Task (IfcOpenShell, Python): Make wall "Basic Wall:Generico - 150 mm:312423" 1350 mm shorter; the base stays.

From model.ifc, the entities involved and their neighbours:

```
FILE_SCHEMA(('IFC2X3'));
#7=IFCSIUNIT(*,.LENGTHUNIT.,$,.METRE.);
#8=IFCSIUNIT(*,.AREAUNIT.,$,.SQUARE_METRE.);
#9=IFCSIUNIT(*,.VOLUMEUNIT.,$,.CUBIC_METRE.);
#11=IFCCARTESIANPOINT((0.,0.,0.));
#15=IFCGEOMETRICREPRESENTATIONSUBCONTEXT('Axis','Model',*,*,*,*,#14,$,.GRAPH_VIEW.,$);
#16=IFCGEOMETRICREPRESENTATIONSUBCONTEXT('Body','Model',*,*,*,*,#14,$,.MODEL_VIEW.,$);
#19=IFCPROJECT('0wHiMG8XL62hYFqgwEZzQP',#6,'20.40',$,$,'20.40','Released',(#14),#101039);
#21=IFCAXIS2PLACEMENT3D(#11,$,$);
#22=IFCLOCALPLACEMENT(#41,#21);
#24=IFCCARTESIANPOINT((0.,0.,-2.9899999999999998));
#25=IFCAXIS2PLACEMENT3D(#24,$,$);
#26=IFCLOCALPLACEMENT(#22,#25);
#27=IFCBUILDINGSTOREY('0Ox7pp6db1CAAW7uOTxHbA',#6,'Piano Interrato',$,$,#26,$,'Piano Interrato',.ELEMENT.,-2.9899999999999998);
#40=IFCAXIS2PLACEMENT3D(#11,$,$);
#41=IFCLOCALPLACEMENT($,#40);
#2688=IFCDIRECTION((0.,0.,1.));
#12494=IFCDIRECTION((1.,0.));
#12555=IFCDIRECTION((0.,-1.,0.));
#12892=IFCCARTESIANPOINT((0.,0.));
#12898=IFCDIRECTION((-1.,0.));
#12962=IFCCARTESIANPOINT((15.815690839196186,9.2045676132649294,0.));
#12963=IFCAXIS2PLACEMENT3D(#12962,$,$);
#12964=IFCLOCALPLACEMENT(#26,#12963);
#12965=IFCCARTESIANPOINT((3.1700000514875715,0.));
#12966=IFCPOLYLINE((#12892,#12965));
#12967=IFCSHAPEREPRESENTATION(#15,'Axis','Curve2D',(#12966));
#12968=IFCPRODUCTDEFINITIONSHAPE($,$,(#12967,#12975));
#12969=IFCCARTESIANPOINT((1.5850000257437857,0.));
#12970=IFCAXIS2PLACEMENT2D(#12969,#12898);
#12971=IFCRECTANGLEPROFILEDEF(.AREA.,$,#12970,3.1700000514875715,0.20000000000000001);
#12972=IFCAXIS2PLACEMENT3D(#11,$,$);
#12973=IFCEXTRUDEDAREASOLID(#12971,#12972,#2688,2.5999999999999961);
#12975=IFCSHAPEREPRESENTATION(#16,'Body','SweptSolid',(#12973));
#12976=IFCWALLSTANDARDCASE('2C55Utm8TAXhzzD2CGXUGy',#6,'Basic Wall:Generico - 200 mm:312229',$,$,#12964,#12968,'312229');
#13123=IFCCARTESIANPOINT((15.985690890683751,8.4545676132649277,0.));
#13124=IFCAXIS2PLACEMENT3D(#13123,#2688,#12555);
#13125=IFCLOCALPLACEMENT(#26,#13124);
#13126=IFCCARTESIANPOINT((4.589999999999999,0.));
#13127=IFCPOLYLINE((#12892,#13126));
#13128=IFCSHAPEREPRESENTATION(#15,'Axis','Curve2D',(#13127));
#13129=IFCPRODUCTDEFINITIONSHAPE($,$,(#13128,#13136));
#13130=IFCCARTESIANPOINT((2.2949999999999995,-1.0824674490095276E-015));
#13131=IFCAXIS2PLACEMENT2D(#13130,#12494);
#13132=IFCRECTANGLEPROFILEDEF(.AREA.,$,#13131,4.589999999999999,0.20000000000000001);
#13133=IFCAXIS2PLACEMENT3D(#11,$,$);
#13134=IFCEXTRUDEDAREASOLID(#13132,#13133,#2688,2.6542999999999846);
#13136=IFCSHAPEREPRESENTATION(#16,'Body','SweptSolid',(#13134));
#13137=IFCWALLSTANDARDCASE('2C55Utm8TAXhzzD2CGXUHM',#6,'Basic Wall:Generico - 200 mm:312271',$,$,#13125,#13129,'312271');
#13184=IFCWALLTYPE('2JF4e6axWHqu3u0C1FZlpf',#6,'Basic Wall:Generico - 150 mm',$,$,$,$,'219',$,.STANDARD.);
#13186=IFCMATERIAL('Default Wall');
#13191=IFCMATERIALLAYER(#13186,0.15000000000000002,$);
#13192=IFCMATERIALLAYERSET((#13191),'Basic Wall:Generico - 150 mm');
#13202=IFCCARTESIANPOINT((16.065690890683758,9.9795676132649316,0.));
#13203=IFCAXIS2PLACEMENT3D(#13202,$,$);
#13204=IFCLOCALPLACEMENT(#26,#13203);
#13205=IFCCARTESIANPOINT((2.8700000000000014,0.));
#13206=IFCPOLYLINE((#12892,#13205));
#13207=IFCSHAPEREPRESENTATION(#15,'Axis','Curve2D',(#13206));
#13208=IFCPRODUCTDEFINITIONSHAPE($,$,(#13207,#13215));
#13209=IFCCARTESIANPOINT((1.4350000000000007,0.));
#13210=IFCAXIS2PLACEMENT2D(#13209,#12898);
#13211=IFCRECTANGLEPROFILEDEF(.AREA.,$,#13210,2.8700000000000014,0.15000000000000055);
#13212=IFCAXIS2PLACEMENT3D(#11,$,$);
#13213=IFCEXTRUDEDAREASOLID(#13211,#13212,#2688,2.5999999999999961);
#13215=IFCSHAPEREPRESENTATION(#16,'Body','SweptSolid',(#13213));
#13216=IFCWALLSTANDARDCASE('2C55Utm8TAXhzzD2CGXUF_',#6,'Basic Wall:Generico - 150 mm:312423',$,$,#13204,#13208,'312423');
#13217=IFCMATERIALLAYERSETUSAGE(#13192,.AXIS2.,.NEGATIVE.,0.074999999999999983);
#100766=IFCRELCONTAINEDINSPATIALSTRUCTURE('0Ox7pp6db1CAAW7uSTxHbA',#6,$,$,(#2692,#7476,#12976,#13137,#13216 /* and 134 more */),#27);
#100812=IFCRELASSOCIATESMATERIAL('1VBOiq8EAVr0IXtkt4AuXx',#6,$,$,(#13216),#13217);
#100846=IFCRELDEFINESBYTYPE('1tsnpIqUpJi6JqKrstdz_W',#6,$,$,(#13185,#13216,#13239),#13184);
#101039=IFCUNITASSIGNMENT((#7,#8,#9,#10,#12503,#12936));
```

```python
import ifcopenshell
import ifcopenshell.geom
import ifcopenshell.util.representation
import ifcopenshell.util.shape
import ifcopenshell.util.unit

model = ifcopenshell.open("model.ifc")
unit_scale = ifcopenshell.util.unit.calculate_unit_scale(model)
settings = ifcopenshell.geom.settings()


def volume(element):
    """Net volume in cubic metres, openings subtracted."""
    shape = ifcopenshell.geom.create_shape(settings, element)
    return ifcopenshell.util.shape.get_volume(shape.geometry)


wall = model.by_guid("2C55Utm8TAXhzzD2CGXUF_")
before = volume(wall)

body = ifcopenshell.util.representation.get_representation(wall, "Model", "Body")
solid = body.Items[0]
old_height = solid.Depth
solid.Depth -= 1.35 / unit_scale
after = volume(wall)

print(f"height {old_height:g} -> {solid.Depth:g}, volume {before:.3f} -> {after:.3f} m3")

model.write("model_v2.ifc")
```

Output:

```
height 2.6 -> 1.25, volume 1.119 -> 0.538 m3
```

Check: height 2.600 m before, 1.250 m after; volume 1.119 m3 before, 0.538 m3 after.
